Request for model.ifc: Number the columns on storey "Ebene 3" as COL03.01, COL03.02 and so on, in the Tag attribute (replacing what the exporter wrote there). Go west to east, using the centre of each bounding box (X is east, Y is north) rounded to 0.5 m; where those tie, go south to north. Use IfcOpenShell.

First a look at what the model holds.

```python
import ifcopenshell
import ifcopenshell.util.element
import ifcopenshell.util.placement

model = ifcopenshell.open("model.ifc")
print(model.schema)
storey = next(s for s in model.by_type("IfcBuildingStorey") if s.Name == "Ebene 3")
columns = [e for e in ifcopenshell.util.element.get_decomposition(storey) if e.is_a("IfcColumn")]
for e in sorted(columns, key=lambda e: e.id()):
    origin = ifcopenshell.util.placement.get_local_placement(e.ObjectPlacement)[:3, 3]
    print(e.id(), e.Tag, e.Name, origin.round(2) + 0.0, sep=" | ")
```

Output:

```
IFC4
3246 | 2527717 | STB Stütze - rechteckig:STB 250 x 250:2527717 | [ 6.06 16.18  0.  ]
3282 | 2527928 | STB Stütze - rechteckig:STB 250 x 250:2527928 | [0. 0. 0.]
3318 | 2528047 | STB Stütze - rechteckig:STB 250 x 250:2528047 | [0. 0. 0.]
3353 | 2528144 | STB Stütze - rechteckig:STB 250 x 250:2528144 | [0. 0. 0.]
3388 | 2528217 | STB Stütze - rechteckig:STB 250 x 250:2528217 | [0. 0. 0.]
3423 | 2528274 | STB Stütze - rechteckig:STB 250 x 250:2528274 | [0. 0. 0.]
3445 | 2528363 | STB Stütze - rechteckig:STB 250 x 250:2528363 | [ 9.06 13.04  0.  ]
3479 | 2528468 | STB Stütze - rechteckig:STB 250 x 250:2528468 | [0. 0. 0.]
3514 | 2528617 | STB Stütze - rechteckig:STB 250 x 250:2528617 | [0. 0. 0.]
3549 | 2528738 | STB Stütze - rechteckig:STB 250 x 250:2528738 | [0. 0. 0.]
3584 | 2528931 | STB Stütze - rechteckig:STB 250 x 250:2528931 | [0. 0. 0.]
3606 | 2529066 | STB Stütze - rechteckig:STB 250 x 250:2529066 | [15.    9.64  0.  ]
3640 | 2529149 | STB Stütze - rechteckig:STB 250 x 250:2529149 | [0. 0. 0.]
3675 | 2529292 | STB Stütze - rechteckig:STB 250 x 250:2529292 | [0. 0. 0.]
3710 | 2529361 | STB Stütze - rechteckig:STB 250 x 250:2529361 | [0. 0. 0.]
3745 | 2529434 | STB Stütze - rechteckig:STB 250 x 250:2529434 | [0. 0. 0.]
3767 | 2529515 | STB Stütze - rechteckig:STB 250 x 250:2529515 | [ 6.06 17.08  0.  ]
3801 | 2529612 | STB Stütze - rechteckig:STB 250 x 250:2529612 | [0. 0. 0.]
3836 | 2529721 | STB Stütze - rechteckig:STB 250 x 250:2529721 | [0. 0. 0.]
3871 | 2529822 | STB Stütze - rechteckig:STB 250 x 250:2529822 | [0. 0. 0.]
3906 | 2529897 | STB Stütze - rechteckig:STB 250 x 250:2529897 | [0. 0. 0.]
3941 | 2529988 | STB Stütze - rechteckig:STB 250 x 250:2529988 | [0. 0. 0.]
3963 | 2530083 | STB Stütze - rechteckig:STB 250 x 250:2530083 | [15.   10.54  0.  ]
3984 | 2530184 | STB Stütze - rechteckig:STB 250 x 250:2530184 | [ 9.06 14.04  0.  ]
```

```python
import ifcopenshell
import ifcopenshell.geom
import ifcopenshell.util.element
import ifcopenshell.util.shape

model = ifcopenshell.open("model.ifc")
settings = ifcopenshell.geom.settings()
settings.set("use-world-coords", True)


def centre(element):
    shape = ifcopenshell.geom.create_shape(settings, element)
    return ifcopenshell.util.shape.get_bbox_centroid(shape.geometry)


storey = next(s for s in model.by_type("IfcBuildingStorey") if s.Name == "Ebene 3")
columns = [e for e in ifcopenshell.util.element.get_decomposition(storey) if e.is_a("IfcColumn")]

# Insertion points can sit at a corner or the storey origin, so sort by the geometry (in metres).
centres = {e: centre(e) for e in columns}
columns.sort(key=lambda e: (round(centres[e][0] / 0.5), centres[e][1]))

for i, e in enumerate(columns, start=1):
    number = f"COL03.{i:02d}"
    e.Tag = number
    print(e.id(), number)

model.write("model-out.ifc")
```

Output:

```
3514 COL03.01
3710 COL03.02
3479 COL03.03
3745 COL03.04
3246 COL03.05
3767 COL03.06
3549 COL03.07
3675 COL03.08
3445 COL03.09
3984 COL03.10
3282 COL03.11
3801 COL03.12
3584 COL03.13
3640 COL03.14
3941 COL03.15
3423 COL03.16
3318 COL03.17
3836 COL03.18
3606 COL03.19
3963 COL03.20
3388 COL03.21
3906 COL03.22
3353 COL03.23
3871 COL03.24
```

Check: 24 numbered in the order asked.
